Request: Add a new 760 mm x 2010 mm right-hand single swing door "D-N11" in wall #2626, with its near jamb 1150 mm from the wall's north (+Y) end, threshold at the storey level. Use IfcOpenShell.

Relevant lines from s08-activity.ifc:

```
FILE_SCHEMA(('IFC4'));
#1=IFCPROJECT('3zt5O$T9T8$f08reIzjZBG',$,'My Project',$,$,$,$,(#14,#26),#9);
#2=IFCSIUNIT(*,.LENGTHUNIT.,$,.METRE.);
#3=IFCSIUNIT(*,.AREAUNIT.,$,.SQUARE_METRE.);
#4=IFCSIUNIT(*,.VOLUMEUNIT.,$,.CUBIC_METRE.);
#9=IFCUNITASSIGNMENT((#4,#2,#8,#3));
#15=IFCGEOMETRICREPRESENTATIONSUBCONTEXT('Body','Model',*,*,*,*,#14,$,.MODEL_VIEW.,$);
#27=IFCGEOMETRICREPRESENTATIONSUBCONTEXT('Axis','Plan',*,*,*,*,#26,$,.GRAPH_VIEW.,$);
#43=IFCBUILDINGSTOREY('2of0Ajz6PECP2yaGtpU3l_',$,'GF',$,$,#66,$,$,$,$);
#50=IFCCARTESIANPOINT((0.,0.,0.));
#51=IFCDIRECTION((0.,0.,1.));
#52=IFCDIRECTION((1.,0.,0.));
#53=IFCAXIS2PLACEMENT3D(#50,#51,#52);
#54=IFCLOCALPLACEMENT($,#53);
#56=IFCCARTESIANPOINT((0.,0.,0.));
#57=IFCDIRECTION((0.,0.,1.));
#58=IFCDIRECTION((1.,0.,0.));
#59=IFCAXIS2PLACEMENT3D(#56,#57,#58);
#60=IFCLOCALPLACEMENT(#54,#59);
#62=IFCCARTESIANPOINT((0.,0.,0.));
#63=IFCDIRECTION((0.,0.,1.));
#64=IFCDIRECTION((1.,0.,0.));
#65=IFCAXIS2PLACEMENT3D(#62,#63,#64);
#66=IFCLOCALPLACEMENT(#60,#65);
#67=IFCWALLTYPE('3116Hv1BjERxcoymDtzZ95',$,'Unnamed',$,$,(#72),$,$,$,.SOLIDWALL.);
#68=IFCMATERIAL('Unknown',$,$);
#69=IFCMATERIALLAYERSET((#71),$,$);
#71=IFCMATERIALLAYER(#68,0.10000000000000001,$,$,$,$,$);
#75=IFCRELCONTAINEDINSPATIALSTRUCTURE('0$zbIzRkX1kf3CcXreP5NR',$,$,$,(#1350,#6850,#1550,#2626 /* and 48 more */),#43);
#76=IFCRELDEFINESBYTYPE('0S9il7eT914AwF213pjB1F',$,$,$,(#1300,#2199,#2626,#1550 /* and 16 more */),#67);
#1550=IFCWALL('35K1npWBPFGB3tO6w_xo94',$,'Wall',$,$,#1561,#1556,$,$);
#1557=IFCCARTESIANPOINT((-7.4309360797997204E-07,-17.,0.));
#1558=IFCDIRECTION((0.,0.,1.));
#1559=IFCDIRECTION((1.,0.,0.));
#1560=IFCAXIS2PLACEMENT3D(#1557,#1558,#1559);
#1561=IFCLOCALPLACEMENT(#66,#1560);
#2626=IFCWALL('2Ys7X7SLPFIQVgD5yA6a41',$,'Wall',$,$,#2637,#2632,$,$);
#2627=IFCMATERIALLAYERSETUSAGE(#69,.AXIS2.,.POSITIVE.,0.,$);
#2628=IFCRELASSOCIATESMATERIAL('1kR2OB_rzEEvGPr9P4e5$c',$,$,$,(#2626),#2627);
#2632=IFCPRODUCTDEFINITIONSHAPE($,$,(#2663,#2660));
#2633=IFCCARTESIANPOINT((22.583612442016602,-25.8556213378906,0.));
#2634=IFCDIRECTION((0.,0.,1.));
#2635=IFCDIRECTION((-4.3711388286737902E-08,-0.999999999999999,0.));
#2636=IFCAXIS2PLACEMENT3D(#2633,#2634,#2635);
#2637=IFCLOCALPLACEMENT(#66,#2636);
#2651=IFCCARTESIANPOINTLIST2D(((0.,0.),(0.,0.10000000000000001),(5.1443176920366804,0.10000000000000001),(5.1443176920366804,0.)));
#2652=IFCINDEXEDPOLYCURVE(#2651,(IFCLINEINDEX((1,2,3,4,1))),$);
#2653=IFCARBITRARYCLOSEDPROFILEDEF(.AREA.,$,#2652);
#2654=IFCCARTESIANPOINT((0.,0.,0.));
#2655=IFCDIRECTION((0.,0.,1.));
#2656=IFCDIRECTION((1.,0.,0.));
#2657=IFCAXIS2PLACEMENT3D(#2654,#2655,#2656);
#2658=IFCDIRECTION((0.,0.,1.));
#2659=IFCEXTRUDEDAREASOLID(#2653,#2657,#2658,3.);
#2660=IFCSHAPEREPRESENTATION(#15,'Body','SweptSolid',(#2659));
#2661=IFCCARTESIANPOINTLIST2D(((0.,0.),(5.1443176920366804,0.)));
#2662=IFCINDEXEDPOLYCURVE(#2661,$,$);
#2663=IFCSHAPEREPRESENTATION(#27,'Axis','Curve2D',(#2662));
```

```python
import numpy as np
import ifcopenshell
import ifcopenshell.api.feature
import ifcopenshell.api.geometry
import ifcopenshell.api.root
import ifcopenshell.api.spatial
import ifcopenshell.geom
import ifcopenshell.util.element
import ifcopenshell.util.placement
import ifcopenshell.util.representation
import ifcopenshell.util.shape
import ifcopenshell.util.unit

model = ifcopenshell.open("s08-activity.ifc")
unit_scale = ifcopenshell.util.unit.calculate_unit_scale(model)
settings = ifcopenshell.geom.settings()


def volume(element):
    """Net volume in cubic metres, openings subtracted."""
    shape = ifcopenshell.geom.create_shape(settings, element)
    return ifcopenshell.util.shape.get_volume(shape.geometry)


wall = model.by_guid("2Ys7X7SLPFIQVgD5yA6a41")
storey = ifcopenshell.util.element.get_container(wall, ifc_class="IfcBuildingStorey")
context = ifcopenshell.util.representation.get_context(model, "Model", "Body", "MODEL_VIEW")
before = volume(wall)

width, height, from_end, sill = 0.76, 2.01, 1.15, 0.0  # metres

# The wall runs along its own X axis, and the end named is its -X end.
wall_shape = ifcopenshell.geom.create_shape(settings, wall)
x, y, z = ifcopenshell.util.shape.get_vertices(wall_shape.geometry).T
start = x.min() + from_end
face, thickness = float(y.min()), float(y.max() - y.min())
wall_matrix = ifcopenshell.util.placement.get_local_placement(wall.ObjectPlacement)
level = ifcopenshell.util.placement.get_local_placement(storey.ObjectPlacement)[2, 3]


def in_wall(x, y):
    """Placement at x, y metres in the wall's axes, at sill height."""
    matrix = wall_matrix.copy()
    matrix[:, 3] = wall_matrix @ np.array([x / unit_scale, y / unit_scale, 0.0, 1.0])
    matrix[2, 3] = level + sill / unit_scale
    return matrix


# Opening: a box that overshoots both wall faces by 50 mm.
opening = ifcopenshell.api.root.create_entity(model, ifc_class="IfcOpeningElement", predefined_type="OPENING")
box = ifcopenshell.api.geometry.add_wall_representation(
    model, context=context, length=width, height=height, thickness=thickness + 0.1
)
ifcopenshell.api.geometry.assign_representation(model, product=opening, representation=box)
ifcopenshell.api.geometry.edit_object_placement(model, product=opening, matrix=in_wall(start, face - 0.05), is_si=False)
ifcopenshell.api.feature.add_feature(model, feature=opening, element=wall)

door = ifcopenshell.api.root.create_entity(model, ifc_class="IfcDoor", name="D-N11", predefined_type="DOOR")
door.OverallWidth, door.OverallHeight = width / unit_scale, height / unit_scale
door.OperationType = "SINGLE_SWING_RIGHT"
body = ifcopenshell.api.geometry.add_door_representation(
    model,
    context=context,
    overall_width=door.OverallWidth,
    overall_height=door.OverallHeight,
    operation_type="SINGLE_SWING_RIGHT",
    lining_properties={"LiningDepth": thickness / unit_scale, "ThresholdDepth": thickness / unit_scale},
)
ifcopenshell.api.geometry.assign_representation(model, product=door, representation=body)
ifcopenshell.api.spatial.assign_container(model, products=[door], relating_structure=storey)
ifcopenshell.api.feature.add_filling(model, opening=opening, element=door)

# The lining spans the wall, so the door starts at the wall face.
ifcopenshell.api.geometry.edit_object_placement(model, product=door, matrix=in_wall(start, face), is_si=False)

after = volume(wall)

print(f"wall volume {before:.3f} -> {after:.3f} m3")

model.write("s08-activity-out.ifc")
```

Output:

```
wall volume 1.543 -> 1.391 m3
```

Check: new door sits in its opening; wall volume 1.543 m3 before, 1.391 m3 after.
